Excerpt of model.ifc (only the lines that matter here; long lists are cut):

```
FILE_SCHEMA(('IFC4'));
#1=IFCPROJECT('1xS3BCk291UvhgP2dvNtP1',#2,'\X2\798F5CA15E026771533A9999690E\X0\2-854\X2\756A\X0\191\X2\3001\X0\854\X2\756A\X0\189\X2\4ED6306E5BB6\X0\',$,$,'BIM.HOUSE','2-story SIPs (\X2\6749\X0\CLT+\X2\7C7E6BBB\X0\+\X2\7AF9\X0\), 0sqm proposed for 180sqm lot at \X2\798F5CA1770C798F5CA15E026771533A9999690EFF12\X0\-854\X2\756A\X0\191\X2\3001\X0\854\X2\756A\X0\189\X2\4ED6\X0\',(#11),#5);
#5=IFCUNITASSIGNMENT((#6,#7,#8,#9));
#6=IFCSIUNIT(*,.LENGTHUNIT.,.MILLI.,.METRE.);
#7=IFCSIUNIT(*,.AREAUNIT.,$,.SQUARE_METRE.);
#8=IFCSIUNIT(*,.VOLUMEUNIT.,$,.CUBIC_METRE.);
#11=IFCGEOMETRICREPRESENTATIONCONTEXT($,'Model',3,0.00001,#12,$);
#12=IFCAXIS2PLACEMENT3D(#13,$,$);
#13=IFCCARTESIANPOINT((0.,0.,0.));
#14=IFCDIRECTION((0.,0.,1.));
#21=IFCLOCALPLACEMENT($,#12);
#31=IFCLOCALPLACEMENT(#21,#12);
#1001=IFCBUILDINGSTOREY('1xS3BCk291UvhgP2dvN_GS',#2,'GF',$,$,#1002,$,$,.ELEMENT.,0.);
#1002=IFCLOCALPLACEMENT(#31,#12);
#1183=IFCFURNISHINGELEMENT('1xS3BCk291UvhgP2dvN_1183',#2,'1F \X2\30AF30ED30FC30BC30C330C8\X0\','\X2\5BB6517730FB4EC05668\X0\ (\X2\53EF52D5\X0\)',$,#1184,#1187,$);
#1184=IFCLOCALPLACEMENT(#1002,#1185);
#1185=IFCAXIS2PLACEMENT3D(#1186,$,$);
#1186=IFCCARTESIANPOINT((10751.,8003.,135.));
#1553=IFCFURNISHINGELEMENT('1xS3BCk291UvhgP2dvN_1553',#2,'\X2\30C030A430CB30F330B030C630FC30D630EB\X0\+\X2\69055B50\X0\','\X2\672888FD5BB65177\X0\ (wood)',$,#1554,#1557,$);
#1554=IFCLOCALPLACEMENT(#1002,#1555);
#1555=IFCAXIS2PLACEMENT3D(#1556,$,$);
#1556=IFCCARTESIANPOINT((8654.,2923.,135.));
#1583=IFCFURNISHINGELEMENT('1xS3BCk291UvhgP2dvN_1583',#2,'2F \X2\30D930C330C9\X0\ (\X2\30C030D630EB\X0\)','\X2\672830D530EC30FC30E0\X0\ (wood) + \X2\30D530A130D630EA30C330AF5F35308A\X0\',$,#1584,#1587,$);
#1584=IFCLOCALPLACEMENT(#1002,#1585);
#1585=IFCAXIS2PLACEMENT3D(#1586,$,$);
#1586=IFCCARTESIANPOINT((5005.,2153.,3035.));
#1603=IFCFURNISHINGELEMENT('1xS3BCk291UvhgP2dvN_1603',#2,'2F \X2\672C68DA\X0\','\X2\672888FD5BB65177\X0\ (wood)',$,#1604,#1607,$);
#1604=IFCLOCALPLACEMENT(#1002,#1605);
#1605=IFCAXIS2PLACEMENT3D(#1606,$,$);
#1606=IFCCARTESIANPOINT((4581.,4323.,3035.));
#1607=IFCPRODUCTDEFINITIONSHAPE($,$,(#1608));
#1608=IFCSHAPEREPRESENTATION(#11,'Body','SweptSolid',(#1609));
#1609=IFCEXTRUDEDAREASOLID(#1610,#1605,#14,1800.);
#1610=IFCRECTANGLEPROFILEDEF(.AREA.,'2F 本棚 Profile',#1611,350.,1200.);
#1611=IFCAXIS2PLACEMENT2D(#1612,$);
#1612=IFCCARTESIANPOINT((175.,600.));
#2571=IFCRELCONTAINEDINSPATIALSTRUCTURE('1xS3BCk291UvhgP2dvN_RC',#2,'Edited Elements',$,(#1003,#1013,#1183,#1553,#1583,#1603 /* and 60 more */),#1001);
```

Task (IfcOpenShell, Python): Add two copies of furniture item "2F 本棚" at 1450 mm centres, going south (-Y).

```python
import numpy as np
import ifcopenshell
import ifcopenshell.api.geometry
import ifcopenshell.api.root
import ifcopenshell.util.element
import ifcopenshell.util.placement

model = ifcopenshell.open("model.ifc")


def reuse_history(source, copy):
    """copy_class also copies each property set's owner history, people and application; keep the originals."""
    for rel in copy.IsDefinedBy:
        if rel.is_a("IfcRelDefinesByProperties") and (history := rel.RelatingPropertyDefinition.OwnerHistory):
            rel.RelatingPropertyDefinition.OwnerHistory = source.OwnerHistory
            ifcopenshell.util.element.remove_deep2(model, history)


source = model.by_guid("1xS3BCk291UvhgP2dvN_1603")
base = ifcopenshell.util.placement.get_local_placement(source.ObjectPlacement)
step = np.array([0.0, -1.0, 0.0]) * 1450.0

for i in range(1, 3):
    copy = ifcopenshell.api.root.copy_class(model, product=source)
    copy.Representation = ifcopenshell.util.element.copy_deep(
        model, source.Representation, exclude=["IfcGeometricRepresentationContext", "IfcRepresentationMap"]
    )
    reuse_history(source, copy)
    matrix = base.copy()
    matrix[:3, 3] += i * step
    print("added at", matrix[:3, 3].round(3) + 0.0)
    ifcopenshell.api.geometry.edit_object_placement(model, product=copy, matrix=matrix, is_si=False)

model.write("model_v2.ifc")
```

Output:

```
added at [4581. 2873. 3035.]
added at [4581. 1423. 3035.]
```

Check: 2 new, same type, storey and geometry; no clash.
